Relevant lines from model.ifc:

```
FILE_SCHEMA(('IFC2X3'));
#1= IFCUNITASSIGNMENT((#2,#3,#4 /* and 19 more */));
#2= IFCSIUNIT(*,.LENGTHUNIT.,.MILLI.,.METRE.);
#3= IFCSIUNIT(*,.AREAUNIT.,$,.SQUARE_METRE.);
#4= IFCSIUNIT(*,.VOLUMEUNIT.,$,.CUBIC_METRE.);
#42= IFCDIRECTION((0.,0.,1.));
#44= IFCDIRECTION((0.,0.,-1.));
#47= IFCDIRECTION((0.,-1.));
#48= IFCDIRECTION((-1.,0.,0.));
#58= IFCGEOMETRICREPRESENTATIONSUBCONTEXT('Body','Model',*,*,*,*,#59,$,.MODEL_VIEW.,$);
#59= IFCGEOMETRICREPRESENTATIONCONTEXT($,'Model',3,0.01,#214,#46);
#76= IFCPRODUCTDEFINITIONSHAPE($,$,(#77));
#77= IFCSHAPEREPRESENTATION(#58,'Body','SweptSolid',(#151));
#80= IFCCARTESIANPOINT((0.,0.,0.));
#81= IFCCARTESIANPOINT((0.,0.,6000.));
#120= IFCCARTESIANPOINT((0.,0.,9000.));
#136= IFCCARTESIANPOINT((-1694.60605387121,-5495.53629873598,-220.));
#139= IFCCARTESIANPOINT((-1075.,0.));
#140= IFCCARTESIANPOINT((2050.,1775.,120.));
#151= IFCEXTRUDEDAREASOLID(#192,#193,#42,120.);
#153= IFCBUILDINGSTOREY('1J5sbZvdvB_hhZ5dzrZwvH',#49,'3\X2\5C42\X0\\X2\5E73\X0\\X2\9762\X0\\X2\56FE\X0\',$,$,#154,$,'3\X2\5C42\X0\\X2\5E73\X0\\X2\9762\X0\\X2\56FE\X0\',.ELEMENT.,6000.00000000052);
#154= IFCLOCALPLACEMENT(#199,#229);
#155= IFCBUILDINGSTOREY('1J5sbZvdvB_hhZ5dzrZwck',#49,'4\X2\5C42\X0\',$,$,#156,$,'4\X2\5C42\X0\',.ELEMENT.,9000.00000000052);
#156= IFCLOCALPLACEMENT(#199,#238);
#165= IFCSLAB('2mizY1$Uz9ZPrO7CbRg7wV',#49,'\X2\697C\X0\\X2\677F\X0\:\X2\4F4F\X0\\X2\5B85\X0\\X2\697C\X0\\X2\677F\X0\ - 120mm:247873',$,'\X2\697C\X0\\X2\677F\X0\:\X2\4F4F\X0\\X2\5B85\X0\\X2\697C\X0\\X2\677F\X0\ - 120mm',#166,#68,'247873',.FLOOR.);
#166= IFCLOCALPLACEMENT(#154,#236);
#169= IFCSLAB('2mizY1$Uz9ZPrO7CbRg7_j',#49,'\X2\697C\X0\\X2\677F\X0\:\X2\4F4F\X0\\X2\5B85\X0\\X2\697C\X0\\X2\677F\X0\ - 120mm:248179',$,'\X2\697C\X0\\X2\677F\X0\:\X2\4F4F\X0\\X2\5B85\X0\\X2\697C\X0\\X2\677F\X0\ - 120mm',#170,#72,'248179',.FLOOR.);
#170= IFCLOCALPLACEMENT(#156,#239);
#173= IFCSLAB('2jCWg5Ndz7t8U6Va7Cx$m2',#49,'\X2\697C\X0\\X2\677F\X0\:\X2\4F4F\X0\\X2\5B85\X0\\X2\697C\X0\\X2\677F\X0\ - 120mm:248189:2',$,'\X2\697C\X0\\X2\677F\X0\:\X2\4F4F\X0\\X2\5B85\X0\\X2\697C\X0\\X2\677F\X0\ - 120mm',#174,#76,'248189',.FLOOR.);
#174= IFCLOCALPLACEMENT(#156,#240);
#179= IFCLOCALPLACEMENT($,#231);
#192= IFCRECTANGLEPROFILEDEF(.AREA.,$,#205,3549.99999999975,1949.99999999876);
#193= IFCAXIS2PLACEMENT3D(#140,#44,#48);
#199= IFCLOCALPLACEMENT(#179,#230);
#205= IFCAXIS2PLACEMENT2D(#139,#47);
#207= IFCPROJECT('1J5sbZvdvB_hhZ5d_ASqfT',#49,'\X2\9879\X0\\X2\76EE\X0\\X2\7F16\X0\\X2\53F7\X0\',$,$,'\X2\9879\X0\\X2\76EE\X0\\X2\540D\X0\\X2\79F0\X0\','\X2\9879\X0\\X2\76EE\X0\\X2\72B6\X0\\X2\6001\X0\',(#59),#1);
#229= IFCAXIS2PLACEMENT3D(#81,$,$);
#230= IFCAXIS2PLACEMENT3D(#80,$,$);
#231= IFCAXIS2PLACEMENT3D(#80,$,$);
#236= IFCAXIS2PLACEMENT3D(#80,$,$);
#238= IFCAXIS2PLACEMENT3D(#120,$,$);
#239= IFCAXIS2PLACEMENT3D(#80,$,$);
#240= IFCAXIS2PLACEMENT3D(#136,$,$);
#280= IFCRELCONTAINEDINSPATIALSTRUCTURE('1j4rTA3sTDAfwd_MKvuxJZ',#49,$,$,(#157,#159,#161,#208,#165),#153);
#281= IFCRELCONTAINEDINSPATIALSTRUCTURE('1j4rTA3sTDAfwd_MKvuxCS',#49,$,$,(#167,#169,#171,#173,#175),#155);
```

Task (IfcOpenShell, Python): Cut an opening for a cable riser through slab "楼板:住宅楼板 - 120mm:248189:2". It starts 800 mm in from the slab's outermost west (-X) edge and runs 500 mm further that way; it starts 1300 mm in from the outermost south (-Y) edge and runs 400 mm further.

```python
import numpy as np
import ifcopenshell
import ifcopenshell.api.feature
import ifcopenshell.api.geometry
import ifcopenshell.api.root
import ifcopenshell.geom
import ifcopenshell.util.placement
import ifcopenshell.util.representation
import ifcopenshell.util.shape
import ifcopenshell.util.unit

model = ifcopenshell.open("model.ifc")
unit_scale = ifcopenshell.util.unit.calculate_unit_scale(model)
settings = ifcopenshell.geom.settings()


def volume(element):
    """Net volume in cubic metres, openings subtracted."""
    shape = ifcopenshell.geom.create_shape(settings, element)
    return ifcopenshell.util.shape.get_volume(shape.geometry)


slab = model.by_id(173)
before = volume(slab)

# Extent in the slab's own axes, in metres. The edges named are its -X and -Y sides.
slab_shape = ifcopenshell.geom.create_shape(settings, slab)
vertices = ifcopenshell.util.shape.get_vertices(slab_shape.geometry)
x_min, y_min, bottom = vertices.min(axis=0)
top = vertices[:, 2].max()

opening = ifcopenshell.api.root.create_entity(model, ifc_class="IfcOpeningElement", name="Cable riser opening")
context = ifcopenshell.util.representation.get_context(model, "Model", "Body", "MODEL_VIEW")
width, depth = 0.5, 0.4
outline = [(0.0, 0.0), (width, 0.0), (width, depth), (0.0, depth), (0.0, 0.0)]
# Overshoot both faces by 50 mm so the cut is clean.
shape = ifcopenshell.api.geometry.add_slab_representation(
    model, context=context, depth=top - bottom + 0.1, polyline=outline
)
ifcopenshell.api.geometry.assign_representation(model, product=opening, representation=shape)

matrix = ifcopenshell.util.placement.get_local_placement(slab.ObjectPlacement)
matrix[:, 3] = matrix @ np.append(np.array([x_min + 0.8, y_min + 1.3, bottom - 0.05]) / unit_scale, 1.0)
ifcopenshell.api.geometry.edit_object_placement(model, product=opening, matrix=matrix, is_si=False)
ifcopenshell.api.feature.add_feature(model, feature=opening, element=slab)

after = volume(slab)

print(f"slab volume {before:.3f} -> {after:.3f} m3")

model.write("model_v2.ifc")
```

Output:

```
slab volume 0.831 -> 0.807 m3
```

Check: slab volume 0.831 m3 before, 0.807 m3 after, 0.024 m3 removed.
